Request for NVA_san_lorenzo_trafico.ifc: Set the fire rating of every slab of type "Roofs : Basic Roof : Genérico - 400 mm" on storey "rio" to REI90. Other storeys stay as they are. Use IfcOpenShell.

First a look at what the model holds.

```python
import ifcopenshell
import ifcopenshell.util.element

model = ifcopenshell.open("NVA_san_lorenzo_trafico.ifc")
print(model.schema)
storey = next(s for s in model.by_type("IfcBuildingStorey") if s.Name == "rio")
slabs = [e for e in ifcopenshell.util.element.get_decomposition(storey) if e.is_a("IfcSlab")]
seen = {}
for e in slabs:
    element_type = ifcopenshell.util.element.get_type(e)
    key = (element_type.Name if element_type != e and element_type else None, ifcopenshell.util.element.get_pset(e, "Pset_SlabCommon", "FireRating"))
    seen[key] = seen.get(key, 0) + 1
for (name, value), count in sorted(seen.items(), key=str):
    print(count, "x", name, "|", value)
```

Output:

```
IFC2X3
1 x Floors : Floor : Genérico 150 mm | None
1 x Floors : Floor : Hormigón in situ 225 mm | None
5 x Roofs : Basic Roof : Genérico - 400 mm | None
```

```python
import ifcopenshell
import ifcopenshell.api.pset
import ifcopenshell.util.element

model = ifcopenshell.open("NVA_san_lorenzo_trafico.ifc")

storey = next(s for s in model.by_type("IfcBuildingStorey") if s.Name == "rio")
slabs = [e for e in ifcopenshell.util.element.get_decomposition(storey) if e.is_a("IfcSlab")]

count = 0
for e in slabs:
    element_type = ifcopenshell.util.element.get_type(e)
    if element_type in (None, e) or element_type.Name != "Roofs : Basic Roof : Genérico - 400 mm":
        continue
    # add_pset returns the element's existing set when there is one.
    pset = ifcopenshell.api.pset.add_pset(model, product=e, name="Pset_SlabCommon")
    ifcopenshell.api.pset.edit_pset(model, pset=pset, properties={"FireRating": "REI90"})
    count += 1

print(count, "slabs updated")

model.write("NVA_san_lorenzo_trafico_edited.ifc")
```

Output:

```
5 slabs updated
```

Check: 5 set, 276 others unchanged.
